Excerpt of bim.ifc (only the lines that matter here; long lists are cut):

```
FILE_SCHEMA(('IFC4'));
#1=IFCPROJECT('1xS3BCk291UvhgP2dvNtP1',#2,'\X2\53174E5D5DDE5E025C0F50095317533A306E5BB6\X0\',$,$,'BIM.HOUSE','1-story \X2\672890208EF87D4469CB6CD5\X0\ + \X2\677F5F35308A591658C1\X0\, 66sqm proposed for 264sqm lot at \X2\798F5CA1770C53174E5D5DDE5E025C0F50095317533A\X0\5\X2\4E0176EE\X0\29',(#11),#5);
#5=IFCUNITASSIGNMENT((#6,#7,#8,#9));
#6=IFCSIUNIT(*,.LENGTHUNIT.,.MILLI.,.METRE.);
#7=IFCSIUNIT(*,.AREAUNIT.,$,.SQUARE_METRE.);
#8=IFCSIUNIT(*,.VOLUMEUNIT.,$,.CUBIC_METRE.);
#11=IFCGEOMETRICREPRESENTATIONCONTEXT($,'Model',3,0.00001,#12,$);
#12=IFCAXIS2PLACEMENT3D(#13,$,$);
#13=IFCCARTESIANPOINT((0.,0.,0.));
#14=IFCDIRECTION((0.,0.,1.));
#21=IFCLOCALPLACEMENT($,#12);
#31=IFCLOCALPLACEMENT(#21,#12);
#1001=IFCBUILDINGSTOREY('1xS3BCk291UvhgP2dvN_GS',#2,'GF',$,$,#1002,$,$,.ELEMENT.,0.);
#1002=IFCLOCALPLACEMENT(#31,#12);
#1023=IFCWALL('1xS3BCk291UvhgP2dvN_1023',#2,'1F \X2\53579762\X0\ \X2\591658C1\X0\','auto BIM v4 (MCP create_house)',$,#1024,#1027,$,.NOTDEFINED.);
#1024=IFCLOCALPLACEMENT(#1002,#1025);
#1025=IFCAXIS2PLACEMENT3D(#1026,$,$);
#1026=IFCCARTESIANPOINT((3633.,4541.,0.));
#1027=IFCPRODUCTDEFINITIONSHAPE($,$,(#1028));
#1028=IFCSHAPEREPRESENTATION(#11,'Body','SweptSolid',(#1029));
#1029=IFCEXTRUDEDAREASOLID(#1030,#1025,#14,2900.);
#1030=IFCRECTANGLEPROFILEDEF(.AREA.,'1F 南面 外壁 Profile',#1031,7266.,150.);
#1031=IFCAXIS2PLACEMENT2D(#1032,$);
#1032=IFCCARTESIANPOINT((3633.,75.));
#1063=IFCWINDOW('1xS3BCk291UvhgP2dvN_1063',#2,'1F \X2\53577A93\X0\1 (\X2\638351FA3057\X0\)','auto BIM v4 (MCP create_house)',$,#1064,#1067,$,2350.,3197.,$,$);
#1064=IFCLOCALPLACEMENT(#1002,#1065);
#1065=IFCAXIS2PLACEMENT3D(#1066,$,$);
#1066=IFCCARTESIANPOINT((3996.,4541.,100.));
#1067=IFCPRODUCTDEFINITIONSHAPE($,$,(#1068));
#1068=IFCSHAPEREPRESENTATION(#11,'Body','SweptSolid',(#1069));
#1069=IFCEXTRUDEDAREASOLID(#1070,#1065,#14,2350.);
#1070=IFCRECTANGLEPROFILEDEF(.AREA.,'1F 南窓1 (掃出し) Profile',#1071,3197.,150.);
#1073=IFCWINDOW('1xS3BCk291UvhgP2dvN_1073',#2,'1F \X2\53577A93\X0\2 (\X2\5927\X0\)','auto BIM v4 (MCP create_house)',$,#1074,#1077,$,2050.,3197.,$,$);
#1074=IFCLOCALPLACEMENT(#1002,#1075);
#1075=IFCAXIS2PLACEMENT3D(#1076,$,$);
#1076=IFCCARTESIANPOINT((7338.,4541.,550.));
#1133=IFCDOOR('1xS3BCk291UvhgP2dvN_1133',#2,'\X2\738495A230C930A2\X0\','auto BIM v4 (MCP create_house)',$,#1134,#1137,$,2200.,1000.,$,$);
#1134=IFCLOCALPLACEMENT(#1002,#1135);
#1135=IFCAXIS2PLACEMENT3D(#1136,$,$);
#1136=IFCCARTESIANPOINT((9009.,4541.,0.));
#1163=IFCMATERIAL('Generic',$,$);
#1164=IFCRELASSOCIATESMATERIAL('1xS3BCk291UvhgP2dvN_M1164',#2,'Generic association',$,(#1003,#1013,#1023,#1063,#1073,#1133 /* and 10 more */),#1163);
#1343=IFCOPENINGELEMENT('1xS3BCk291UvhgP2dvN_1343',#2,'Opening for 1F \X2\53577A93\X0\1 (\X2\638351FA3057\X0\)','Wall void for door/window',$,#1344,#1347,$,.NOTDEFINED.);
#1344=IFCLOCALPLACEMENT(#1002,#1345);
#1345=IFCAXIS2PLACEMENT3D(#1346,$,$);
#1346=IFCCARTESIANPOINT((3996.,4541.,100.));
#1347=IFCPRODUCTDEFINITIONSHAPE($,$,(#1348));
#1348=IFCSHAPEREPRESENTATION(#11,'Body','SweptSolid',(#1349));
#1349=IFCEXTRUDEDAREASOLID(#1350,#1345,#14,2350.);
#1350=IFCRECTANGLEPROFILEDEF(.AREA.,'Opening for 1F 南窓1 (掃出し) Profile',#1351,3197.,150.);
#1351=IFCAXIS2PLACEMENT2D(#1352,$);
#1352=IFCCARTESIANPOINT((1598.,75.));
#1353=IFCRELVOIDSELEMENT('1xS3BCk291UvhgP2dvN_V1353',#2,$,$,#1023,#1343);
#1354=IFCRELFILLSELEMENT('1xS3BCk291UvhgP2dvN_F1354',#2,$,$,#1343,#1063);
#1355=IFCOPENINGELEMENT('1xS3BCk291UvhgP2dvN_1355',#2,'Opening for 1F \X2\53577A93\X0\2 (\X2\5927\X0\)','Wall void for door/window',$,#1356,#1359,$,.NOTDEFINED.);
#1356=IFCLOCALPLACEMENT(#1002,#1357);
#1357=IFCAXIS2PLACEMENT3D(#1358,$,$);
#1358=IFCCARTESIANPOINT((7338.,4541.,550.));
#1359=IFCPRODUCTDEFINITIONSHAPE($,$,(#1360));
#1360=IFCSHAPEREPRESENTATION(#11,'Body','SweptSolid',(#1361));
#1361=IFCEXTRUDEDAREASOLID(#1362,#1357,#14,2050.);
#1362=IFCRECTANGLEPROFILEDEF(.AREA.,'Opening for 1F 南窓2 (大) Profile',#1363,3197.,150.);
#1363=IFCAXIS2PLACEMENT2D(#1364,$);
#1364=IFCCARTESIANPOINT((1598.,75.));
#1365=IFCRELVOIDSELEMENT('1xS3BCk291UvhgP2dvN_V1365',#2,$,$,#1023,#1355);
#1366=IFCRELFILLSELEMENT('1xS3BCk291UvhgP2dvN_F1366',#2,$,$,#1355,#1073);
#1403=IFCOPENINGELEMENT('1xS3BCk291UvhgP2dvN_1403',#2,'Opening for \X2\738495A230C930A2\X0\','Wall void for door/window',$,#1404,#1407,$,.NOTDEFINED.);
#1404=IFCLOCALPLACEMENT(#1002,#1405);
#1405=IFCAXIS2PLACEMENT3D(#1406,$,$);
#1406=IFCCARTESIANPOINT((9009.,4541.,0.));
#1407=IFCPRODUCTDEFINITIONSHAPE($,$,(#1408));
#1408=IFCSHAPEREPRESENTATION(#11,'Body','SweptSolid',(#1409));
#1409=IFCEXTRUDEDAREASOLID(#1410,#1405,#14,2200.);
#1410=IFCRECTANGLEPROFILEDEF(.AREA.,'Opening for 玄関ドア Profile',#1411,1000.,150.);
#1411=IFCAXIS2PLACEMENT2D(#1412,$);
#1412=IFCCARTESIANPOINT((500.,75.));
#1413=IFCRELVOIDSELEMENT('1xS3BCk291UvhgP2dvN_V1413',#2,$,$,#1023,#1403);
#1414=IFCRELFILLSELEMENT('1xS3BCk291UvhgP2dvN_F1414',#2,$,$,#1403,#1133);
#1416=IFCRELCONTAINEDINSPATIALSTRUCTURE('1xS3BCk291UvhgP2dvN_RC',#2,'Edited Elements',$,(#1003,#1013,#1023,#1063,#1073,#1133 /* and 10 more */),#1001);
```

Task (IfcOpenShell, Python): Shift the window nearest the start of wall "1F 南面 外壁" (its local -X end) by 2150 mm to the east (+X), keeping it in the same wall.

```python
import ifcopenshell
import ifcopenshell.api.geometry
import ifcopenshell.util.placement
import ifcopenshell.util.unit

model = ifcopenshell.open("bim.ifc")
unit_scale = ifcopenshell.util.unit.calculate_unit_scale(model)

window = model.by_guid("1xS3BCk291UvhgP2dvN_1063")
opening = window.FillsVoids[0].RelatingOpeningElement
wall = opening.VoidsElements[0].RelatingBuildingElement

wall_matrix = ifcopenshell.util.placement.get_local_placement(wall.ObjectPlacement)
shift = wall_matrix[:3, 0] * 2.15 / unit_scale
before = ifcopenshell.util.placement.get_local_placement(window.ObjectPlacement)[:3, 3].copy()

# The window is not placed relative to its opening, so move both.
for product in (opening, window):
    matrix = ifcopenshell.util.placement.get_local_placement(product.ObjectPlacement)
    matrix[:3, 3] += shift
    ifcopenshell.api.geometry.edit_object_placement(model, product=product, matrix=matrix, is_si=False)

after = ifcopenshell.util.placement.get_local_placement(window.ObjectPlacement)[:3, 3]
print("window moved by", (after - before).round(3) + 0.0)

model.write("bim_edited.ifc")
```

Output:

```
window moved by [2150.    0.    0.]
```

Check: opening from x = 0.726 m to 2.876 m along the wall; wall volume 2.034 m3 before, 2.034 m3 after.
